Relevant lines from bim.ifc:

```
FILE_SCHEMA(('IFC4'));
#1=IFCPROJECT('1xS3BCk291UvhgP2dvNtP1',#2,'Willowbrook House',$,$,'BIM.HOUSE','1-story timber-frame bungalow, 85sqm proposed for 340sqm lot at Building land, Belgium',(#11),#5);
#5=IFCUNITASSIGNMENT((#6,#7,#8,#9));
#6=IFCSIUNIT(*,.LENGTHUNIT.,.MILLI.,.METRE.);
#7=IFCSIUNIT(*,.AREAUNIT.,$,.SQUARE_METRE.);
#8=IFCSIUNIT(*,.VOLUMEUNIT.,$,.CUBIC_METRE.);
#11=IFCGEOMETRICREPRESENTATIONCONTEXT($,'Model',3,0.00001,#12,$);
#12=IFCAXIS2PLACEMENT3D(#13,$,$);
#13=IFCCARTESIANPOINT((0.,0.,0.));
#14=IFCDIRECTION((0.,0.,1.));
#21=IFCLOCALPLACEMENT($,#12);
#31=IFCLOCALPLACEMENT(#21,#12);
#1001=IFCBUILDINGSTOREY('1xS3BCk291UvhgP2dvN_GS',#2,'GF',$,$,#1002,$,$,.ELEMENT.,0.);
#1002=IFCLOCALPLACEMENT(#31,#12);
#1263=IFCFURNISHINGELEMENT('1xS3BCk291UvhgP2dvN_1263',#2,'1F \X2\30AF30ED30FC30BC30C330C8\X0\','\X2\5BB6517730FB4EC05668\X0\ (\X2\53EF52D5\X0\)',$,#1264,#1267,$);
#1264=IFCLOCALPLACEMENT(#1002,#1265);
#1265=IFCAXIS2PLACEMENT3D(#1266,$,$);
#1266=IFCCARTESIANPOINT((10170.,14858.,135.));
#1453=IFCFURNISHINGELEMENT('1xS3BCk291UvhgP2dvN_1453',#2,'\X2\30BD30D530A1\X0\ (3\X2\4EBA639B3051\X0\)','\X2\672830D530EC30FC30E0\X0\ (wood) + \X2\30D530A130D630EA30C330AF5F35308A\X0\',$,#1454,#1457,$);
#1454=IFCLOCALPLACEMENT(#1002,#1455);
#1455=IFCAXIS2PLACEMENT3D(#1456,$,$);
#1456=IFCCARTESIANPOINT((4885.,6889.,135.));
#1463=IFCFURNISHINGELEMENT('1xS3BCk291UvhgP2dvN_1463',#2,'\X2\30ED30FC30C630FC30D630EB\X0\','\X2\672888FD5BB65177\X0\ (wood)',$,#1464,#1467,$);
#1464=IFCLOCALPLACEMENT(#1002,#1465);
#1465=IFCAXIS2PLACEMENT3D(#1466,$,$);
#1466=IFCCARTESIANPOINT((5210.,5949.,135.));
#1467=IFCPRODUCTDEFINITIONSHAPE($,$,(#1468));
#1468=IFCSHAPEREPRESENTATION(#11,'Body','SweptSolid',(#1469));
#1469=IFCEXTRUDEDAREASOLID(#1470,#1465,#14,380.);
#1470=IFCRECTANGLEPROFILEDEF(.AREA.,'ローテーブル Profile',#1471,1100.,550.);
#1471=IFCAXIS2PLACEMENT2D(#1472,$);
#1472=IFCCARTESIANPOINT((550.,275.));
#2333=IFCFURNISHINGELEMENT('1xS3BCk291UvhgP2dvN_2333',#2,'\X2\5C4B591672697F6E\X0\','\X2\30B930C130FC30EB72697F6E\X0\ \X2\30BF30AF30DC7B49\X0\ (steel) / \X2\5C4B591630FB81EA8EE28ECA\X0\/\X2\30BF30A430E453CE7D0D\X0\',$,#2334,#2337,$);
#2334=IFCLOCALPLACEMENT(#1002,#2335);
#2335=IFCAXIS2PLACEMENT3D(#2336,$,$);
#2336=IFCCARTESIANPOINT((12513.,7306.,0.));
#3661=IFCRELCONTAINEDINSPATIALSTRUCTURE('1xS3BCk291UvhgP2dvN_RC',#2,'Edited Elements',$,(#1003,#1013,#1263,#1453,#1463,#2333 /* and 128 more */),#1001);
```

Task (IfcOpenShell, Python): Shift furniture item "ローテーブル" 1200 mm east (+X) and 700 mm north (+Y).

```python
import ifcopenshell
import ifcopenshell.api.geometry
import ifcopenshell.util.placement
import ifcopenshell.util.unit

model = ifcopenshell.open("bim.ifc")
unit_scale = ifcopenshell.util.unit.calculate_unit_scale(model)

item = model.by_id(1463)
matrix = ifcopenshell.util.placement.get_local_placement(item.ObjectPlacement)
matrix[0, 3] += 1.2 / unit_scale
matrix[1, 3] += 0.7 / unit_scale
ifcopenshell.api.geometry.edit_object_placement(model, product=item, matrix=matrix, is_si=False)

print(ifcopenshell.util.placement.get_local_placement(item.ObjectPlacement).round(3) + 0.0)

model.write("bim_updated.ifc")
```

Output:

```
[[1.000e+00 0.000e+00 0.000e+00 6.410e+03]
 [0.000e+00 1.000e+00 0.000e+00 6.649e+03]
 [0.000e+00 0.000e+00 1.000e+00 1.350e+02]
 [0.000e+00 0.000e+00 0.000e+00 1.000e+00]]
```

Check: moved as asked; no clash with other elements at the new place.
